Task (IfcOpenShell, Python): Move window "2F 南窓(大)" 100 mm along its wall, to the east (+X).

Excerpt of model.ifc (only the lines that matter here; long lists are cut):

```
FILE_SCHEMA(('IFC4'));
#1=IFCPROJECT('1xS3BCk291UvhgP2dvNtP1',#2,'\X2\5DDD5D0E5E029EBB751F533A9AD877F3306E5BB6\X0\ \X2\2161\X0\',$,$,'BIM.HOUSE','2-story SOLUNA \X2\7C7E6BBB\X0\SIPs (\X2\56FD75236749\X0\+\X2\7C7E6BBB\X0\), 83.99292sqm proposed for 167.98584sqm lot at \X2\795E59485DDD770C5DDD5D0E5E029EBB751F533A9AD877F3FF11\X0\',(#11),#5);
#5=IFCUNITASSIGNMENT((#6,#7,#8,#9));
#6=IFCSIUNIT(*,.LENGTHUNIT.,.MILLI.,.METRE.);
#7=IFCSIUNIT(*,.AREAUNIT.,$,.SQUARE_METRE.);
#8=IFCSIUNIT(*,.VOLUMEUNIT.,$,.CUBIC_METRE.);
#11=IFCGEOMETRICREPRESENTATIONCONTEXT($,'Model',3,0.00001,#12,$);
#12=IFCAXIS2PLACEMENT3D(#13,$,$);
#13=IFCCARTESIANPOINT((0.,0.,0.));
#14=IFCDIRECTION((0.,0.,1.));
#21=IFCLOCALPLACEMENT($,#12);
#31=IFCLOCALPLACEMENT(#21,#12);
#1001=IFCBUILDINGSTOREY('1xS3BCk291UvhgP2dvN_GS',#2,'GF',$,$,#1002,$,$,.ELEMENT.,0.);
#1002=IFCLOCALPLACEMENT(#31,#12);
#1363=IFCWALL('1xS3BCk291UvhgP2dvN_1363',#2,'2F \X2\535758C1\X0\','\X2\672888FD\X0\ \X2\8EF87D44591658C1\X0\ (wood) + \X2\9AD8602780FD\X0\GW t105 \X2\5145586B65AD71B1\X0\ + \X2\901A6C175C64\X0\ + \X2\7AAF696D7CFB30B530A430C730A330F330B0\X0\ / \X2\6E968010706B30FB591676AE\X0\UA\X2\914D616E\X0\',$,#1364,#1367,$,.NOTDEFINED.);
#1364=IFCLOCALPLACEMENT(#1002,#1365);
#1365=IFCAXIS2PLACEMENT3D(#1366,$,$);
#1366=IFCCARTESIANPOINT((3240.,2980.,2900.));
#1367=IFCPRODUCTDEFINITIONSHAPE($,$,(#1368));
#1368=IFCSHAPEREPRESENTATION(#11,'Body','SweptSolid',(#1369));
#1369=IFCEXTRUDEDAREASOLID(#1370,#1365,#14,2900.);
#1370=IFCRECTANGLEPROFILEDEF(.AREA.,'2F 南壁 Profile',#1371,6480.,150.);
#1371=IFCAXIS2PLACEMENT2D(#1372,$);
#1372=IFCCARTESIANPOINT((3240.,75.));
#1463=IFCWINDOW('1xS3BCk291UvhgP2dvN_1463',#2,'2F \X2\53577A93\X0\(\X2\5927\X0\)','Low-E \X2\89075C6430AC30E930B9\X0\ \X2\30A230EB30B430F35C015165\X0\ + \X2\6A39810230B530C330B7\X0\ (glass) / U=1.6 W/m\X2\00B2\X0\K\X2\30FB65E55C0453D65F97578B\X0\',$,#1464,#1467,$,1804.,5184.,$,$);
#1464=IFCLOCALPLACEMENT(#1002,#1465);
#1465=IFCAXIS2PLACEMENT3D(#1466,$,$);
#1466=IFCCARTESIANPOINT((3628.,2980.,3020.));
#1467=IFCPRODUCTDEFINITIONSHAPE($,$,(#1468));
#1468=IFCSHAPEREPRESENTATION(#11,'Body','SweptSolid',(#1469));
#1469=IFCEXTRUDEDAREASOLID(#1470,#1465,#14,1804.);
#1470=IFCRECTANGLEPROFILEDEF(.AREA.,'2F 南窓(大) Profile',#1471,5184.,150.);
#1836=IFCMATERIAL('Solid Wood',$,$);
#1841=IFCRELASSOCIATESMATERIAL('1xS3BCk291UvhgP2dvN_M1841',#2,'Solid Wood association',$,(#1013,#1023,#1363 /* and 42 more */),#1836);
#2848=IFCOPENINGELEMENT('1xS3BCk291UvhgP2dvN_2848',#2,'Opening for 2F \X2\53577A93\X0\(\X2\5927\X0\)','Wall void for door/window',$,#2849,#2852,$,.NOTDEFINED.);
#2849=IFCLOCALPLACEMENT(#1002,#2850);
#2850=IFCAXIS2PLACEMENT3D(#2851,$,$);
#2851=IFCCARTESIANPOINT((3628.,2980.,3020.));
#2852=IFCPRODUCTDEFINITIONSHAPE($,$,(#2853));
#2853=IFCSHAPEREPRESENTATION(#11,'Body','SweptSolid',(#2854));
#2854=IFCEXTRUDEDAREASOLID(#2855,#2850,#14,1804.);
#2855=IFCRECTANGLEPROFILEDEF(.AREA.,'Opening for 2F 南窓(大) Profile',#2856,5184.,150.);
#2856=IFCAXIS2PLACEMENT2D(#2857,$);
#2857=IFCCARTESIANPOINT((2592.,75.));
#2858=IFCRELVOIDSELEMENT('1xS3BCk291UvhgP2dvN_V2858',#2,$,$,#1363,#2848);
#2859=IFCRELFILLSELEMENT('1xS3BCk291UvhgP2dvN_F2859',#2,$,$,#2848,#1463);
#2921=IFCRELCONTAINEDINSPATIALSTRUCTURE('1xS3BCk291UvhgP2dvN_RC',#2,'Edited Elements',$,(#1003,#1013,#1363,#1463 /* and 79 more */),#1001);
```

```python
import ifcopenshell
import ifcopenshell.api.geometry
import ifcopenshell.util.placement
import ifcopenshell.util.unit

model = ifcopenshell.open("model.ifc")
unit_scale = ifcopenshell.util.unit.calculate_unit_scale(model)

window = model.by_guid("1xS3BCk291UvhgP2dvN_1463")
opening = window.FillsVoids[0].RelatingOpeningElement
wall = opening.VoidsElements[0].RelatingBuildingElement

wall_matrix = ifcopenshell.util.placement.get_local_placement(wall.ObjectPlacement)
shift = wall_matrix[:3, 0] * 0.1 / unit_scale
before = ifcopenshell.util.placement.get_local_placement(window.ObjectPlacement)[:3, 3].copy()

# The window is not placed relative to its opening, so move both.
for product in (opening, window):
    matrix = ifcopenshell.util.placement.get_local_placement(product.ObjectPlacement)
    matrix[:3, 3] += shift
    ifcopenshell.api.geometry.edit_object_placement(model, product=product, matrix=matrix, is_si=False)

after = ifcopenshell.util.placement.get_local_placement(window.ObjectPlacement)[:3, 3]
print("window moved by", (after - before).round(3) + 0.0)

model.write("model_edited.ifc")
```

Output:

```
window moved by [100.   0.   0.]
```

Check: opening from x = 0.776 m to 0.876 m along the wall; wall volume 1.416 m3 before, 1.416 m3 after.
